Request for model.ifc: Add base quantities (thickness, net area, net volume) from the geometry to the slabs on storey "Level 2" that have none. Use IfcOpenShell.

First a look at what the model holds.

```python
import ifcopenshell
import ifcopenshell.util.element
import ifcopenshell.util.unit

model = ifcopenshell.open("model.ifc")
print(model.schema)
for unit_type in ("LENGTHUNIT", "AREAUNIT", "VOLUMEUNIT"):
    print(unit_type, ifcopenshell.util.unit.calculate_unit_scale(model, unit_type))
storey = next(s for s in model.by_type("IfcBuildingStorey") if s.Name == "Level 2")
slabs = [e for e in ifcopenshell.util.element.get_decomposition(storey) if e.is_a("IfcSlab")]
for e in sorted(slabs, key=lambda e: e.id()):
    print(e.id(), e.is_a(), e.Name, list(ifcopenshell.util.element.get_psets(e, qtos_only=True)), sep=" | ")
```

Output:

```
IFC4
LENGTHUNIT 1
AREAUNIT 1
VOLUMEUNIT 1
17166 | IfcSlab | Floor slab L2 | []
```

```python
import ifcopenshell
import ifcopenshell.api.pset
import ifcopenshell.geom
import ifcopenshell.util.element
import ifcopenshell.util.shape
import ifcopenshell.util.unit

model = ifcopenshell.open("model.ifc")
unit_scale = ifcopenshell.util.unit.calculate_unit_scale(model)
area_scale = ifcopenshell.util.unit.calculate_unit_scale(model, "AREAUNIT")
volume_scale = ifcopenshell.util.unit.calculate_unit_scale(model, "VOLUMEUNIT")
settings = ifcopenshell.geom.settings()

storey = next(s for s in model.by_type("IfcBuildingStorey") if s.Name == "Level 2")
slabs = [e for e in ifcopenshell.util.element.get_decomposition(storey) if e.is_a("IfcSlab")]

for e in sorted(slabs, key=lambda e: e.id()):
    if ifcopenshell.util.element.get_psets(e, qtos_only=True, should_inherit=False):
        continue
    # Geometry comes back in metres, in the element's own axes.
    shape = ifcopenshell.geom.create_shape(settings, e)
    values = {
        "Width": ifcopenshell.util.shape.get_z(shape.geometry) / unit_scale,
        "NetArea": ifcopenshell.util.shape.get_footprint_area(shape.geometry) / area_scale,
        "NetVolume": ifcopenshell.util.shape.get_volume(shape.geometry) / volume_scale,
    }
    qto = ifcopenshell.api.pset.add_qto(model, product=e, name="Qto_SlabBaseQuantities")
    ifcopenshell.api.pset.edit_qto(model, qto=qto, properties=values)
    print(e.id(), {k: round(v, 3) for k, v in values.items()})

model.write("model_updated.ifc")
```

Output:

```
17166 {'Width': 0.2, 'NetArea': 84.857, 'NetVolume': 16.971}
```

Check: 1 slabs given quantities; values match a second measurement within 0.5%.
